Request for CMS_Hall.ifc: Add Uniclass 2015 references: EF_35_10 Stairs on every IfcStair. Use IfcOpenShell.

First a look at what the model holds.

```python
import ifcopenshell

model = ifcopenshell.open("CMS_Hall.ifc")
print(model.schema)
print("classifications:", [c.Name for c in model.by_type("IfcClassification")])
for ifc_class in ("IfcDoor", "IfcRoof", "IfcStair", "IfcWall", "IfcWindow"):
    print(ifc_class, len(model.by_type(ifc_class)))
```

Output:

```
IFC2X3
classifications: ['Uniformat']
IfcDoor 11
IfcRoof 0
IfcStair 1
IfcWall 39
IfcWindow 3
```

```python
import ifcopenshell
import ifcopenshell.api.classification

model = ifcopenshell.open("CMS_Hall.ifc")

# IFC2X3 requires Source and Edition and has no link from the project to the system.
system = model.create_entity("IfcClassification", Source="NBS", Edition="2015", Name="Uniclass 2015")

codes = {
    "IfcStair": ("EF_35_10", "Stairs"),
}
for ifc_class, (code, name) in codes.items():
    products = model.by_type(ifc_class)
    ifcopenshell.api.classification.add_reference(
        model, products=products, classification=system, identification=code, name=name
    )
    print(code, len(products))

model.write("CMS_Hall-out.ifc")
```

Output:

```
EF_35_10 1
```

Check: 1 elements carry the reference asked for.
